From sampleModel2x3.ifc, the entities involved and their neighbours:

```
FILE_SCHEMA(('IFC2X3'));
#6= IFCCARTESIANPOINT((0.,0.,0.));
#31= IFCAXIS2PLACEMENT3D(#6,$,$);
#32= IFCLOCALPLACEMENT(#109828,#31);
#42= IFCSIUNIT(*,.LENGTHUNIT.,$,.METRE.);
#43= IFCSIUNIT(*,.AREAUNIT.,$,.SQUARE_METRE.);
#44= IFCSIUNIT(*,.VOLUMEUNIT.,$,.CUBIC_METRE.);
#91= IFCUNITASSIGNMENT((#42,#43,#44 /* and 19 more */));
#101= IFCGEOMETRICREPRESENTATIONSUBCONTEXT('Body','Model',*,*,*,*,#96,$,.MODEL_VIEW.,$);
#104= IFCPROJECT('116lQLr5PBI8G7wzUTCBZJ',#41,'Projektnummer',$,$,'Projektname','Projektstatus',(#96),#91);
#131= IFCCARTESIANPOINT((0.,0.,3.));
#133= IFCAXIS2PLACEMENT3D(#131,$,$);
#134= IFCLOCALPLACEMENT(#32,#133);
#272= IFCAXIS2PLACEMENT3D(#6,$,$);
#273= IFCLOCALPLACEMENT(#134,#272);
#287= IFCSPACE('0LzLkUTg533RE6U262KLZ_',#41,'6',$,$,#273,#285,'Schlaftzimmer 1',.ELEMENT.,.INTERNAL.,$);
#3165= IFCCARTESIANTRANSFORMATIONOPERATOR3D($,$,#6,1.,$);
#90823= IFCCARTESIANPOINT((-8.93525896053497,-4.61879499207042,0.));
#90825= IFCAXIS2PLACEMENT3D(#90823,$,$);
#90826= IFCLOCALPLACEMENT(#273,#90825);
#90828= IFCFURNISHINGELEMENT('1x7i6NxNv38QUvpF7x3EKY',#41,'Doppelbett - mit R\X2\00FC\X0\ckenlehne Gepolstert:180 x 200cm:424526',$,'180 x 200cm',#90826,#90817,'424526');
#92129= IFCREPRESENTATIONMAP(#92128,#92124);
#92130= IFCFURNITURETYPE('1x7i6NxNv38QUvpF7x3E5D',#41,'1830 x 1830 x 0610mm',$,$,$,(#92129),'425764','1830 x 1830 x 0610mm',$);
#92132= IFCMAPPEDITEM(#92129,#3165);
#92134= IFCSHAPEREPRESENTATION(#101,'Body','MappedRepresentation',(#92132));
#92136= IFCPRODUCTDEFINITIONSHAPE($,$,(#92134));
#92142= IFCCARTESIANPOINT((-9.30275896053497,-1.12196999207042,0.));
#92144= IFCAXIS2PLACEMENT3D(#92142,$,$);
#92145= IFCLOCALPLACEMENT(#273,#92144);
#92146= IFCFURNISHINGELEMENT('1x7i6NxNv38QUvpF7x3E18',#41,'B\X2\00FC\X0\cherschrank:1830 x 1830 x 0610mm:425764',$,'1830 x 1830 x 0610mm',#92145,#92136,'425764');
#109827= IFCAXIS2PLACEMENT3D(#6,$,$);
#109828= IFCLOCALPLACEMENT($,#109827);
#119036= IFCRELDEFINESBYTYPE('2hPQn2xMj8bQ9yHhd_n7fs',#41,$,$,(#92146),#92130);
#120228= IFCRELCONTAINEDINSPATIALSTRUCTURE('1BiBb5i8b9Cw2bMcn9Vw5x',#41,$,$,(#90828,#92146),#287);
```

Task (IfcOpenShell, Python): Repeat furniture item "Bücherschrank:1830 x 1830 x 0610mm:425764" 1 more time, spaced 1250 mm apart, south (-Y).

```python
import numpy as np
import ifcopenshell
import ifcopenshell.api.geometry
import ifcopenshell.api.root
import ifcopenshell.util.element
import ifcopenshell.util.placement

model = ifcopenshell.open("sampleModel2x3.ifc")

source = model.by_guid("1x7i6NxNv38QUvpF7x3E18")
base = ifcopenshell.util.placement.get_local_placement(source.ObjectPlacement)
step = np.array([0.0, -1.0, 0.0]) * 1.25

for i in range(1, 2):
    copy = ifcopenshell.api.root.copy_class(model, product=source)
    copy.Representation = ifcopenshell.util.element.copy_deep(
        model, source.Representation, exclude=["IfcGeometricRepresentationContext", "IfcRepresentationMap"]
    )
    copy.Name = "Bücherschrank:1830 x 1830 x 0610mm"
    copy.Tag = None
    matrix = base.copy()
    matrix[:3, 3] += i * step
    print("added at", matrix[:3, 3].round(3) + 0.0)
    ifcopenshell.api.geometry.edit_object_placement(model, product=copy, matrix=matrix, is_si=False)

model.write("sampleModel2x3_edited.ifc")
```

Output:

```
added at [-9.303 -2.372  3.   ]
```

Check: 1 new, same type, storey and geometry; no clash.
